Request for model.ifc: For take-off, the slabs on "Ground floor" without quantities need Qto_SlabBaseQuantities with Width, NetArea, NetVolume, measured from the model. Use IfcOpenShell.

First a look at what the model holds.

```python
import ifcopenshell
import ifcopenshell.util.element
import ifcopenshell.util.unit

model = ifcopenshell.open("model.ifc")
print(model.schema)
for unit_type in ("LENGTHUNIT", "AREAUNIT", "VOLUMEUNIT"):
    print(unit_type, ifcopenshell.util.unit.calculate_unit_scale(model, unit_type))
storey = next(s for s in model.by_type("IfcBuildingStorey") if s.Name == "Ground floor")
slabs = [e for e in ifcopenshell.util.element.get_decomposition(storey) if e.is_a("IfcSlab")]
for e in sorted(slabs, key=lambda e: e.id()):
    print(e.id(), e.is_a(), e.Name, list(ifcopenshell.util.element.get_psets(e, qtos_only=True)), sep=" | ")
```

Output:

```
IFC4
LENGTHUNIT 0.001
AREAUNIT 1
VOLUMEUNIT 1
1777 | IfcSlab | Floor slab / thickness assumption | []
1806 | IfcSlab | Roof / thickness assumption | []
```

```python
import ifcopenshell
import ifcopenshell.api.pset
import ifcopenshell.geom
import ifcopenshell.util.element
import ifcopenshell.util.shape
import ifcopenshell.util.unit

model = ifcopenshell.open("model.ifc")
unit_scale = ifcopenshell.util.unit.calculate_unit_scale(model)
area_scale = ifcopenshell.util.unit.calculate_unit_scale(model, "AREAUNIT")
volume_scale = ifcopenshell.util.unit.calculate_unit_scale(model, "VOLUMEUNIT")
settings = ifcopenshell.geom.settings()

storey = next(s for s in model.by_type("IfcBuildingStorey") if s.Name == "Ground floor")
slabs = [e for e in ifcopenshell.util.element.get_decomposition(storey) if e.is_a("IfcSlab")]

for e in sorted(slabs, key=lambda e: e.id()):
    if ifcopenshell.util.element.get_psets(e, qtos_only=True, should_inherit=False):
        continue
    # Geometry comes back in metres, in the element's own axes.
    shape = ifcopenshell.geom.create_shape(settings, e)
    values = {
        "Width": ifcopenshell.util.shape.get_z(shape.geometry) / unit_scale,
        "NetArea": ifcopenshell.util.shape.get_footprint_area(shape.geometry) / area_scale,
        "NetVolume": ifcopenshell.util.shape.get_volume(shape.geometry) / volume_scale,
    }
    qto = ifcopenshell.api.pset.add_qto(model, product=e, name="Qto_SlabBaseQuantities")
    ifcopenshell.api.pset.edit_qto(model, qto=qto, properties=values)
    print(e.id(), {k: round(v, 3) for k, v in values.items()})

model.write("model_updated.ifc")
```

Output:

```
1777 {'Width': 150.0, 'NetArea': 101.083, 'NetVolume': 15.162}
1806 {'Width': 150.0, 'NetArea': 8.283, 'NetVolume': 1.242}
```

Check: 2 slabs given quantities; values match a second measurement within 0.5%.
